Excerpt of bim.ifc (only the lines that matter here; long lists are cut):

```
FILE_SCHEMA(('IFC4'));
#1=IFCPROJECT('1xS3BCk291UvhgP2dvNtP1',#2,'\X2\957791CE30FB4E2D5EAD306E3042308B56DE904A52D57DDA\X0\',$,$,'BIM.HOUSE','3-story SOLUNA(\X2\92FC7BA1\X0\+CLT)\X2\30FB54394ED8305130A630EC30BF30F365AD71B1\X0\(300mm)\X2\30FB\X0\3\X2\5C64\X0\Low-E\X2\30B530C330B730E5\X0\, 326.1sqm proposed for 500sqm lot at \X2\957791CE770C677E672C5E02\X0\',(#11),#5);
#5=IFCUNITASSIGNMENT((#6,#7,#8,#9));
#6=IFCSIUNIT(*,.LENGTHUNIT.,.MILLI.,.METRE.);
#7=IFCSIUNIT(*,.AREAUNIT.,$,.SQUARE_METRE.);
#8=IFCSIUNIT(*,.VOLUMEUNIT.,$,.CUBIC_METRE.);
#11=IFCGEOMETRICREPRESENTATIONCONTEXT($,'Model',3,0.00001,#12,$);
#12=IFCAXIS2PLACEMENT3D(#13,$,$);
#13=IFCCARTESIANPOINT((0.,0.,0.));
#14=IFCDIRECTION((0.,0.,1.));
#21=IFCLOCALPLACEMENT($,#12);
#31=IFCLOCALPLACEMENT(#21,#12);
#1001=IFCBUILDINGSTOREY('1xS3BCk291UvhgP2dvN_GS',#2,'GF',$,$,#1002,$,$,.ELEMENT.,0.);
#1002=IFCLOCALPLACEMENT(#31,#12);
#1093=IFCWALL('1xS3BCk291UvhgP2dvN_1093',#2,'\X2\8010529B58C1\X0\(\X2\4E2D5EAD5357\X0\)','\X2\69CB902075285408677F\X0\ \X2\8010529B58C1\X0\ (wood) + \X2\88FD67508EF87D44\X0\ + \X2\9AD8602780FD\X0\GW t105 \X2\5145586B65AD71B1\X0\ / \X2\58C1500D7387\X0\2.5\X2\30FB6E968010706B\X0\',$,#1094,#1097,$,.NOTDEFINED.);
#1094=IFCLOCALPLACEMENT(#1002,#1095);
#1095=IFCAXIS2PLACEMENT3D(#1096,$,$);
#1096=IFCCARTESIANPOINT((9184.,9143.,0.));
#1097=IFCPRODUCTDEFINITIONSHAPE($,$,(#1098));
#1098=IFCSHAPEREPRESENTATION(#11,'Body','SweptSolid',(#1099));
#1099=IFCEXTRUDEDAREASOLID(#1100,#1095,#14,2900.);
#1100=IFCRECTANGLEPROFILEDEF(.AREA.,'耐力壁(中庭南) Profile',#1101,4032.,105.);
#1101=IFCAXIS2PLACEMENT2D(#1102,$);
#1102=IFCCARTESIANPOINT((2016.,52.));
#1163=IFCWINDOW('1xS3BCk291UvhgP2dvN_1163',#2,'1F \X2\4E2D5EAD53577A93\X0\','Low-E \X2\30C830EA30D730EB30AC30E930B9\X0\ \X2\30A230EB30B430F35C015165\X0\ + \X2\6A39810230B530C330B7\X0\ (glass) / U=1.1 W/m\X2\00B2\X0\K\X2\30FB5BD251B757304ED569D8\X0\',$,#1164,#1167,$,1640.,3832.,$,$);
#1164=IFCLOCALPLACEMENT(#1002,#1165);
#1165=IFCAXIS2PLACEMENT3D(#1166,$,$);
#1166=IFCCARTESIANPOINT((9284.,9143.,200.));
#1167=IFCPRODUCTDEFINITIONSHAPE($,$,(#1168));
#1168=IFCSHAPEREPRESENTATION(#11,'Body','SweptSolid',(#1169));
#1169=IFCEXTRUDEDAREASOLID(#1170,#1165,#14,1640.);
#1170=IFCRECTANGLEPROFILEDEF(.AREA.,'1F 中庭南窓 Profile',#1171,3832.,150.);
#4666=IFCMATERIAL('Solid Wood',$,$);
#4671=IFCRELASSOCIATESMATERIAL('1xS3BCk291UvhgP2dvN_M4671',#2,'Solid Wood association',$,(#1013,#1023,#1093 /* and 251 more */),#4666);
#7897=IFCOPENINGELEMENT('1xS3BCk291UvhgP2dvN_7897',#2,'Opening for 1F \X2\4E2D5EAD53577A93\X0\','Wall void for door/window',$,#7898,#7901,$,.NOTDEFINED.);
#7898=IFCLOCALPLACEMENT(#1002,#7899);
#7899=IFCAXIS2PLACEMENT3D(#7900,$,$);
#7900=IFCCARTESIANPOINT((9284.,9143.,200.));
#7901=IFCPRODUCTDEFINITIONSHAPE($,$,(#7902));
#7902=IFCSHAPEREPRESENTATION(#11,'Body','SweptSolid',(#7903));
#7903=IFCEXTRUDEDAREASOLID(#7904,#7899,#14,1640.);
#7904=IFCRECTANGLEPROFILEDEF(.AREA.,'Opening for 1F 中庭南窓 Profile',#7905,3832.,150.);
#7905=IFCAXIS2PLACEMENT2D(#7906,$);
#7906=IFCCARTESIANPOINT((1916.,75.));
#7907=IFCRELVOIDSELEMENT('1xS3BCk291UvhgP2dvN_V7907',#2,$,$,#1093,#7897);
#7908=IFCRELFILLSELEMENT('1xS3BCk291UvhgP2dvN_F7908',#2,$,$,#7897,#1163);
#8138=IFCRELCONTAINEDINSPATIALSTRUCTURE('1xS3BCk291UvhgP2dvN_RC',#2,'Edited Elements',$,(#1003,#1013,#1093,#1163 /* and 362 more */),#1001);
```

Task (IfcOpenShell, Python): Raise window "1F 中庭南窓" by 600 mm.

```python
import numpy as np
import ifcopenshell
import ifcopenshell.api.geometry
import ifcopenshell.util.placement
import ifcopenshell.util.unit

model = ifcopenshell.open("bim.ifc")
unit_scale = ifcopenshell.util.unit.calculate_unit_scale(model)

window = model.by_guid("1xS3BCk291UvhgP2dvN_1163")
opening = window.FillsVoids[0].RelatingOpeningElement
dz = 0.6 / unit_scale

shift = np.array([0.0, 0.0, dz])
# The window is not placed relative to its opening, so move both.
for product in (opening, window):
    matrix = ifcopenshell.util.placement.get_local_placement(product.ObjectPlacement)
    matrix[:3, 3] += shift
    ifcopenshell.api.geometry.edit_object_placement(model, product=product, matrix=matrix, is_si=False)

print(f"moved by {dz * unit_scale:+.3f} m")

model.write("bim_updated.ifc")
```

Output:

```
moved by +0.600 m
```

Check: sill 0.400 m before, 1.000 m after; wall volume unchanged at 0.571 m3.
